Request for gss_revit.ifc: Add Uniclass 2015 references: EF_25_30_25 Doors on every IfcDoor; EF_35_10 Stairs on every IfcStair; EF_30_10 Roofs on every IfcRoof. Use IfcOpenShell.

First a look at what the model holds.

```python
import ifcopenshell

model = ifcopenshell.open("gss_revit.ifc")
print(model.schema)
print("classifications:", [c.Name for c in model.by_type("IfcClassification")])
for ifc_class in ("IfcDoor", "IfcRoof", "IfcStair", "IfcWall", "IfcWindow"):
    print(ifc_class, len(model.by_type(ifc_class)))
```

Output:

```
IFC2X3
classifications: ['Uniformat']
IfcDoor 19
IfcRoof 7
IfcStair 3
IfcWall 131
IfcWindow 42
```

```python
import ifcopenshell
import ifcopenshell.api.classification

model = ifcopenshell.open("gss_revit.ifc")

# IFC2X3 requires Source and Edition and has no link from the project to the system.
system = model.create_entity("IfcClassification", Source="NBS", Edition="2015", Name="Uniclass 2015")

codes = {
    "IfcDoor": ("EF_25_30_25", "Doors"),
    "IfcStair": ("EF_35_10", "Stairs"),
    "IfcRoof": ("EF_30_10", "Roofs"),
}
for ifc_class, (code, name) in codes.items():
    products = model.by_type(ifc_class)
    ifcopenshell.api.classification.add_reference(
        model, products=products, classification=system, identification=code, name=name
    )
    print(code, len(products))

model.write("gss_revit_updated.ifc")
```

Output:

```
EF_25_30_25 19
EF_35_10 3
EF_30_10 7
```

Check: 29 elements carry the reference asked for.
